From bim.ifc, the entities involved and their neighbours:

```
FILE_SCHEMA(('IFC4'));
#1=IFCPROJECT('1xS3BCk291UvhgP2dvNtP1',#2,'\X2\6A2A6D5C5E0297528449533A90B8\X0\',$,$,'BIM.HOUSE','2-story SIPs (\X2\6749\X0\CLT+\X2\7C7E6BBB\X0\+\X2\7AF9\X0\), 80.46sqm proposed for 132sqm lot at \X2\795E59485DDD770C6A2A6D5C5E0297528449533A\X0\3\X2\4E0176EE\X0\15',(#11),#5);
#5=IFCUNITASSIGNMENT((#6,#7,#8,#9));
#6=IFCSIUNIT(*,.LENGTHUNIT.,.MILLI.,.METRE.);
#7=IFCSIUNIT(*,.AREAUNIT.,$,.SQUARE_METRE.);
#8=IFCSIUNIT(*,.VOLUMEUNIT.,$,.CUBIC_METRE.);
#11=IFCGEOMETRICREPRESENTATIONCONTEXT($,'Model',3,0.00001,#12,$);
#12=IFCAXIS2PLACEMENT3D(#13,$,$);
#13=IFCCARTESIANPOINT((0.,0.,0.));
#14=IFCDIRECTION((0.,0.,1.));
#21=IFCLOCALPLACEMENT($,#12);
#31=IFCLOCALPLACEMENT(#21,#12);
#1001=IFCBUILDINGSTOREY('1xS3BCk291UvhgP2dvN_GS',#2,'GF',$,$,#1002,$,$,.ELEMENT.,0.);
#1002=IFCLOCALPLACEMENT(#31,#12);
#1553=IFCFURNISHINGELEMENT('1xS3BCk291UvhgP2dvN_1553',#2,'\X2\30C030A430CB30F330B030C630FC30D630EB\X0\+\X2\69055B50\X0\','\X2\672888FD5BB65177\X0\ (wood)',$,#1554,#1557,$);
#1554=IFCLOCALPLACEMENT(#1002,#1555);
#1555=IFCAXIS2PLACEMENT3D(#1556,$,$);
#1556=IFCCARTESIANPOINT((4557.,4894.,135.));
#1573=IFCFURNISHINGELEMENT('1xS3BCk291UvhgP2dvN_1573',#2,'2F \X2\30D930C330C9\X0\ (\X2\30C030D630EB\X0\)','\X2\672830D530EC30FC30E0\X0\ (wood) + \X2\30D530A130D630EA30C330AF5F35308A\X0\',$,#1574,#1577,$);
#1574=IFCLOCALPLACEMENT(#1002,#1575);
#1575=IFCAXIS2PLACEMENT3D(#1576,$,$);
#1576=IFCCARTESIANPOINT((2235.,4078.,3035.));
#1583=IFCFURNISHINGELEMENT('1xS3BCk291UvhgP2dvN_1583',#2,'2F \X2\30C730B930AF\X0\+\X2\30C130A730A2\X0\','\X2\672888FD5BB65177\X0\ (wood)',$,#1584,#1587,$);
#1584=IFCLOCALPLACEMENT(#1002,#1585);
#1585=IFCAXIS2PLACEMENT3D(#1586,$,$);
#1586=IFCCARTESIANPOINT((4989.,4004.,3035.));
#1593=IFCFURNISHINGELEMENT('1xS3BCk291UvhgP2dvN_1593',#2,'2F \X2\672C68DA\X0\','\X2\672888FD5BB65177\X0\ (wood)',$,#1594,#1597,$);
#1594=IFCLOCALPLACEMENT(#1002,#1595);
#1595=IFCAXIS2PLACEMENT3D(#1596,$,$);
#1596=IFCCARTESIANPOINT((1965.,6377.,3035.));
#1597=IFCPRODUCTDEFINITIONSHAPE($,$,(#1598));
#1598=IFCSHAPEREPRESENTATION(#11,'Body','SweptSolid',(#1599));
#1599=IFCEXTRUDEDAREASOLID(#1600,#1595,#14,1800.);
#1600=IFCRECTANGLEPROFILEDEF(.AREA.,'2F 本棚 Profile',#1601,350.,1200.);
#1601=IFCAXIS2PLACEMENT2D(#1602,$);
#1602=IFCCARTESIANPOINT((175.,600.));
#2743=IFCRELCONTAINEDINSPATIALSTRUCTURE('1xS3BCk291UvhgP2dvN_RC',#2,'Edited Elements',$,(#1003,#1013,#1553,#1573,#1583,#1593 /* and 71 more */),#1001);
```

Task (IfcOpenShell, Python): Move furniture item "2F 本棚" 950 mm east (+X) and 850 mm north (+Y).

```python
import ifcopenshell
import ifcopenshell.api.geometry
import ifcopenshell.util.placement
import ifcopenshell.util.unit

model = ifcopenshell.open("bim.ifc")
unit_scale = ifcopenshell.util.unit.calculate_unit_scale(model)

item = model.by_guid("1xS3BCk291UvhgP2dvN_1593")
matrix = ifcopenshell.util.placement.get_local_placement(item.ObjectPlacement)
matrix[0, 3] += 0.95 / unit_scale
matrix[1, 3] += 0.85 / unit_scale
ifcopenshell.api.geometry.edit_object_placement(model, product=item, matrix=matrix, is_si=False)

print(ifcopenshell.util.placement.get_local_placement(item.ObjectPlacement).round(3) + 0.0)

model.write("bim_edited.ifc")
```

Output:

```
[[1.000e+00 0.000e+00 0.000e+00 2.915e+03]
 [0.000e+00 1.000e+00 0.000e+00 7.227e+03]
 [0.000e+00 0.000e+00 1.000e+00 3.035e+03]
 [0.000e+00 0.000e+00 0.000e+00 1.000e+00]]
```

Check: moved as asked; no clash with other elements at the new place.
